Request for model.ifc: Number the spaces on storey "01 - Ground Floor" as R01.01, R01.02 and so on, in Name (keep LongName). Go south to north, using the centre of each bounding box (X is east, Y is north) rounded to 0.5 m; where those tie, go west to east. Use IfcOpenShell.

First a look at what the model holds.

```python
import ifcopenshell
import ifcopenshell.util.element
import ifcopenshell.util.placement

model = ifcopenshell.open("model.ifc")
print(model.schema)
storey = next(s for s in model.by_type("IfcBuildingStorey") if s.Name == "01 - Ground Floor")
spaces = [e for e in ifcopenshell.util.element.get_decomposition(storey) if e.is_a("IfcSpace")]
for e in sorted(spaces, key=lambda e: e.id()):
    origin = ifcopenshell.util.placement.get_local_placement(e.ObjectPlacement)[:3, 3]
    print(e.id(), e.Name, e.LongName, origin.round(2) + 0.0, sep=" | ")
```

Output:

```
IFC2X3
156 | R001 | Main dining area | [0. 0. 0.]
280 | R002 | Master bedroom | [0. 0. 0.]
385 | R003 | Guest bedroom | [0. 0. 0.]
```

```python
import ifcopenshell
import ifcopenshell.geom
import ifcopenshell.util.element
import ifcopenshell.util.shape

model = ifcopenshell.open("model.ifc")
settings = ifcopenshell.geom.settings()
settings.set("use-world-coords", True)


def centre(element):
    shape = ifcopenshell.geom.create_shape(settings, element)
    return ifcopenshell.util.shape.get_bbox_centroid(shape.geometry)


storey = next(s for s in model.by_type("IfcBuildingStorey") if s.Name == "01 - Ground Floor")
spaces = [e for e in ifcopenshell.util.element.get_decomposition(storey) if e.is_a("IfcSpace")]

# Insertion points can sit at a corner or the storey origin, so sort by the geometry (in metres).
centres = {e: centre(e) for e in spaces}
spaces.sort(key=lambda e: (round(centres[e][1] / 0.5), centres[e][0]))

for i, e in enumerate(spaces, start=1):
    number = f"R01.{i:02d}"
    e.Name = number
    print(e.id(), number)

model.write("model_v2.ifc")
```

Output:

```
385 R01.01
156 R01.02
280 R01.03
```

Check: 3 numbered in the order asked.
